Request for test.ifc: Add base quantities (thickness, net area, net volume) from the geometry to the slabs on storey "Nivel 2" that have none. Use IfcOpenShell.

First a look at what the model holds.

```python
import ifcopenshell
import ifcopenshell.util.element
import ifcopenshell.util.unit

model = ifcopenshell.open("test.ifc")
print(model.schema)
for unit_type in ("LENGTHUNIT", "AREAUNIT", "VOLUMEUNIT"):
    print(unit_type, ifcopenshell.util.unit.calculate_unit_scale(model, unit_type))
storey = next(s for s in model.by_type("IfcBuildingStorey") if s.Name == "Nivel 2")
slabs = [e for e in ifcopenshell.util.element.get_decomposition(storey) if e.is_a("IfcSlab")]
for e in sorted(slabs, key=lambda e: e.id()):
    print(e.id(), e.is_a(), e.Name, list(ifcopenshell.util.element.get_psets(e, qtos_only=True)), sep=" | ")
```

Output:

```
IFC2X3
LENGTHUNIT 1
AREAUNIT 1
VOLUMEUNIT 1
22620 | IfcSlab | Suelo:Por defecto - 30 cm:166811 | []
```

```python
import ifcopenshell
import ifcopenshell.api.pset
import ifcopenshell.geom
import ifcopenshell.util.element
import ifcopenshell.util.shape
import ifcopenshell.util.unit

model = ifcopenshell.open("test.ifc")
unit_scale = ifcopenshell.util.unit.calculate_unit_scale(model)
area_scale = ifcopenshell.util.unit.calculate_unit_scale(model, "AREAUNIT")
volume_scale = ifcopenshell.util.unit.calculate_unit_scale(model, "VOLUMEUNIT")
settings = ifcopenshell.geom.settings()

storey = next(s for s in model.by_type("IfcBuildingStorey") if s.Name == "Nivel 2")
slabs = [e for e in ifcopenshell.util.element.get_decomposition(storey) if e.is_a("IfcSlab")]

for e in sorted(slabs, key=lambda e: e.id()):
    if ifcopenshell.util.element.get_psets(e, qtos_only=True, should_inherit=False):
        continue
    # Geometry comes back in metres, in the element's own axes.
    shape = ifcopenshell.geom.create_shape(settings, e)
    values = {
        "Width": ifcopenshell.util.shape.get_z(shape.geometry) / unit_scale,
        "NetArea": ifcopenshell.util.shape.get_footprint_area(shape.geometry) / area_scale,
        "NetVolume": ifcopenshell.util.shape.get_volume(shape.geometry) / volume_scale,
    }
    qto = ifcopenshell.api.pset.add_qto(model, product=e, name="BaseQuantities")
    ifcopenshell.api.pset.edit_qto(model, qto=qto, properties=values)
    print(e.id(), {k: round(v, 3) for k, v in values.items()})

model.write("test_rev.ifc")
```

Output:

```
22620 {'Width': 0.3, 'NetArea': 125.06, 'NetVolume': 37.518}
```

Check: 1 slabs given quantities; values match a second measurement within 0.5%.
